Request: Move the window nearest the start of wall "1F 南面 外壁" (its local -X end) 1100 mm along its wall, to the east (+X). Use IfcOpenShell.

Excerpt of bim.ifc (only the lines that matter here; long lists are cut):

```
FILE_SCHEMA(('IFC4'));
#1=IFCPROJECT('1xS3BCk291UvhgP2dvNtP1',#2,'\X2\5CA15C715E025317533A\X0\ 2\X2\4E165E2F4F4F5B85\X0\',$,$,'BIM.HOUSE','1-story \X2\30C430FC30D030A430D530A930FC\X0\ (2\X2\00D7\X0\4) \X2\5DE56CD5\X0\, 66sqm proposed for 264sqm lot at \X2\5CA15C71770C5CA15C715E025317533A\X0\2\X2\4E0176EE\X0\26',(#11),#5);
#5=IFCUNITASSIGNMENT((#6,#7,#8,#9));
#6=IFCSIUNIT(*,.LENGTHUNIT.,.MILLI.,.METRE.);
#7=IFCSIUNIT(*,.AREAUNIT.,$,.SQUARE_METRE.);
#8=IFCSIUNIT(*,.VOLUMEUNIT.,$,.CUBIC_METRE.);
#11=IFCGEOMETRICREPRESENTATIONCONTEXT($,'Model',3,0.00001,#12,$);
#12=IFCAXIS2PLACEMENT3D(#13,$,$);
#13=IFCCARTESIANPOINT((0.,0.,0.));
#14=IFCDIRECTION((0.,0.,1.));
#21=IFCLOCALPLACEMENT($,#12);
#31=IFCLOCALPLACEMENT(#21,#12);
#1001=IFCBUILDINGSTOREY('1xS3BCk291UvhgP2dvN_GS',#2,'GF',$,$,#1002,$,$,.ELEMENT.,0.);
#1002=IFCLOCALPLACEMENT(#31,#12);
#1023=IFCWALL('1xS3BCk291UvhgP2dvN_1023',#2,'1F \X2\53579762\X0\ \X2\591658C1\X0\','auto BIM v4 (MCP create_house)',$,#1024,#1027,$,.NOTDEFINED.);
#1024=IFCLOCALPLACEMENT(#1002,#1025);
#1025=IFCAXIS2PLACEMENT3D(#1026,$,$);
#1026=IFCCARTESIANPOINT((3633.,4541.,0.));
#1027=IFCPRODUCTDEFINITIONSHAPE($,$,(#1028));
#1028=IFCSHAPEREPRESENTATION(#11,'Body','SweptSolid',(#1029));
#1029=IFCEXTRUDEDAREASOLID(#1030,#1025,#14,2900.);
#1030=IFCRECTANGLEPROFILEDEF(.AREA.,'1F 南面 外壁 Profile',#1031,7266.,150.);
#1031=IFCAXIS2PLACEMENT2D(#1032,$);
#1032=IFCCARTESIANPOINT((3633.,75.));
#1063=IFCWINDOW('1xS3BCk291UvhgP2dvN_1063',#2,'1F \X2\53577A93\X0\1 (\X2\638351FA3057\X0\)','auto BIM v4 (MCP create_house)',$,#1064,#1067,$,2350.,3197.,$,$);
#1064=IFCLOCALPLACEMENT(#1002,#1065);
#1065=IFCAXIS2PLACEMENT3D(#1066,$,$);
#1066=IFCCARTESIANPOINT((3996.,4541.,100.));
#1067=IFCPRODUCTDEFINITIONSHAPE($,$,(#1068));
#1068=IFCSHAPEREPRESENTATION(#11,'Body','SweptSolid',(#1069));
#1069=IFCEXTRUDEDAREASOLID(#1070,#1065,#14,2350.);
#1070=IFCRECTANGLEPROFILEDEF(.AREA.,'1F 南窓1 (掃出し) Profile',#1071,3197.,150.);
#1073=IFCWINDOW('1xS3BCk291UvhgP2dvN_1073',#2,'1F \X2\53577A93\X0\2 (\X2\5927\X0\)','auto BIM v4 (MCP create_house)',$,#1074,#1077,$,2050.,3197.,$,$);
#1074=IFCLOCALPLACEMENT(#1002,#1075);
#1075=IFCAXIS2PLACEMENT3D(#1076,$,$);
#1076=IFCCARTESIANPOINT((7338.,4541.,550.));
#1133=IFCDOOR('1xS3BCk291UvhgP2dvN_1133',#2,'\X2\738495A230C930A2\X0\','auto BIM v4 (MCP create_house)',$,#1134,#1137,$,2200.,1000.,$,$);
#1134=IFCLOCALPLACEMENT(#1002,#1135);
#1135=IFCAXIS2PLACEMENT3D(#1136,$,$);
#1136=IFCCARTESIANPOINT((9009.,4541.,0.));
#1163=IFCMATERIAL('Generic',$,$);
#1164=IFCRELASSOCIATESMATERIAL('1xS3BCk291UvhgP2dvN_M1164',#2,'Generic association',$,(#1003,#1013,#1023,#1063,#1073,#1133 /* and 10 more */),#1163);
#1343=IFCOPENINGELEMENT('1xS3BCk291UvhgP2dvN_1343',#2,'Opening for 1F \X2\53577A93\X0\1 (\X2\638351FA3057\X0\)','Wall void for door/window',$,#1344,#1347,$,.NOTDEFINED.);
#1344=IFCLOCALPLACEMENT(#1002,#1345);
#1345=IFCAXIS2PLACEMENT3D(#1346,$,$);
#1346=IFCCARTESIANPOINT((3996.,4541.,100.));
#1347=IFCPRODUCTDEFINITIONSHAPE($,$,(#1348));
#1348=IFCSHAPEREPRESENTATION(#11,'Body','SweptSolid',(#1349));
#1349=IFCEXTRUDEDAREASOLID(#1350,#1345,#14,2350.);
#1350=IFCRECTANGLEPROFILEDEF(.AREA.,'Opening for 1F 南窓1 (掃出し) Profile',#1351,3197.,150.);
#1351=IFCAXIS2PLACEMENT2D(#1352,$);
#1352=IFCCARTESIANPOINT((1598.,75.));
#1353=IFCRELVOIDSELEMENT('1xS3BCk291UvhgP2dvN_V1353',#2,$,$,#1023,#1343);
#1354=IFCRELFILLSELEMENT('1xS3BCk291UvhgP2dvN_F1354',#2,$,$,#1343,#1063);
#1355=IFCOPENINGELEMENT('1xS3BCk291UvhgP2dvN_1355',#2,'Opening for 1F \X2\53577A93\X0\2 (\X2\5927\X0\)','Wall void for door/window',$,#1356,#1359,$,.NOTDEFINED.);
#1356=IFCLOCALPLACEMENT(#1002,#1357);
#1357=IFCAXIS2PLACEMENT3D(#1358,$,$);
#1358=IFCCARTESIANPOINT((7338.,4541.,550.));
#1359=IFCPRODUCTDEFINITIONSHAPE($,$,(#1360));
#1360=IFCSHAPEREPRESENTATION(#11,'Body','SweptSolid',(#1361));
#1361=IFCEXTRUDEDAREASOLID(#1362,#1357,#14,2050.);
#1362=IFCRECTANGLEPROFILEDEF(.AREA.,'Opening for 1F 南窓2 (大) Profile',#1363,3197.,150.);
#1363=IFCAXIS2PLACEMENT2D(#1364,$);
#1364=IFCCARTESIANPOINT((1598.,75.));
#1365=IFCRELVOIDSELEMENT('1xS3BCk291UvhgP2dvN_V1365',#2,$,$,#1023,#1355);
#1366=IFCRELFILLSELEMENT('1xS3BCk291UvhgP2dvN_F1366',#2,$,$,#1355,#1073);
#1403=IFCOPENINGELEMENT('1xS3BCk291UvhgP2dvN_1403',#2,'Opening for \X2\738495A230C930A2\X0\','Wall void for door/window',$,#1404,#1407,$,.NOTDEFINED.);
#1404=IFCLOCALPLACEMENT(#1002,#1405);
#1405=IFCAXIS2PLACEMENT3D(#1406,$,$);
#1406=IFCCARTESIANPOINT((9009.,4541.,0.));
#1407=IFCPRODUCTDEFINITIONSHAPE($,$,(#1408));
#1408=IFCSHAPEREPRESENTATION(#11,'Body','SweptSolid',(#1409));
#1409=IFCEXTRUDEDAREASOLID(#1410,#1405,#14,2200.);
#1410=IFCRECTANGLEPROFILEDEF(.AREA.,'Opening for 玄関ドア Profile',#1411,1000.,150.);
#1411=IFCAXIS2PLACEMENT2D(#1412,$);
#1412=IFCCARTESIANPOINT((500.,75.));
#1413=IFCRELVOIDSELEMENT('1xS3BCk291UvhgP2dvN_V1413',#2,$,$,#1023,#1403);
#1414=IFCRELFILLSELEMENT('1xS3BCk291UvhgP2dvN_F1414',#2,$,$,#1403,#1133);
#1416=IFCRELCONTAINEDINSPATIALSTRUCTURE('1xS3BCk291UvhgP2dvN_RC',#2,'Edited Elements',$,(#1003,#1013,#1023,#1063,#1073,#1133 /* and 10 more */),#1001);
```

```python
import ifcopenshell
import ifcopenshell.api.geometry
import ifcopenshell.util.placement

model = ifcopenshell.open("bim.ifc")

window = model.by_guid("1xS3BCk291UvhgP2dvN_1063")
opening = window.FillsVoids[0].RelatingOpeningElement
wall = opening.VoidsElements[0].RelatingBuildingElement

wall_matrix = ifcopenshell.util.placement.get_local_placement(wall.ObjectPlacement)
shift = wall_matrix[:3, 0] * 1100.0
before = ifcopenshell.util.placement.get_local_placement(window.ObjectPlacement)[:3, 3].copy()

# The window is not placed relative to its opening, so move both.
for product in (opening, window):
    matrix = ifcopenshell.util.placement.get_local_placement(product.ObjectPlacement)
    matrix[:3, 3] += shift
    ifcopenshell.api.geometry.edit_object_placement(model, product=product, matrix=matrix, is_si=False)

after = ifcopenshell.util.placement.get_local_placement(window.ObjectPlacement)[:3, 3]
print("window moved by", (after - before).round(3) + 0.0)

model.write("bim_edited.ifc")
```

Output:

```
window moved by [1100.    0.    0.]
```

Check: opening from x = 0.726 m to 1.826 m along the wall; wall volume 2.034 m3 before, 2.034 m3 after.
